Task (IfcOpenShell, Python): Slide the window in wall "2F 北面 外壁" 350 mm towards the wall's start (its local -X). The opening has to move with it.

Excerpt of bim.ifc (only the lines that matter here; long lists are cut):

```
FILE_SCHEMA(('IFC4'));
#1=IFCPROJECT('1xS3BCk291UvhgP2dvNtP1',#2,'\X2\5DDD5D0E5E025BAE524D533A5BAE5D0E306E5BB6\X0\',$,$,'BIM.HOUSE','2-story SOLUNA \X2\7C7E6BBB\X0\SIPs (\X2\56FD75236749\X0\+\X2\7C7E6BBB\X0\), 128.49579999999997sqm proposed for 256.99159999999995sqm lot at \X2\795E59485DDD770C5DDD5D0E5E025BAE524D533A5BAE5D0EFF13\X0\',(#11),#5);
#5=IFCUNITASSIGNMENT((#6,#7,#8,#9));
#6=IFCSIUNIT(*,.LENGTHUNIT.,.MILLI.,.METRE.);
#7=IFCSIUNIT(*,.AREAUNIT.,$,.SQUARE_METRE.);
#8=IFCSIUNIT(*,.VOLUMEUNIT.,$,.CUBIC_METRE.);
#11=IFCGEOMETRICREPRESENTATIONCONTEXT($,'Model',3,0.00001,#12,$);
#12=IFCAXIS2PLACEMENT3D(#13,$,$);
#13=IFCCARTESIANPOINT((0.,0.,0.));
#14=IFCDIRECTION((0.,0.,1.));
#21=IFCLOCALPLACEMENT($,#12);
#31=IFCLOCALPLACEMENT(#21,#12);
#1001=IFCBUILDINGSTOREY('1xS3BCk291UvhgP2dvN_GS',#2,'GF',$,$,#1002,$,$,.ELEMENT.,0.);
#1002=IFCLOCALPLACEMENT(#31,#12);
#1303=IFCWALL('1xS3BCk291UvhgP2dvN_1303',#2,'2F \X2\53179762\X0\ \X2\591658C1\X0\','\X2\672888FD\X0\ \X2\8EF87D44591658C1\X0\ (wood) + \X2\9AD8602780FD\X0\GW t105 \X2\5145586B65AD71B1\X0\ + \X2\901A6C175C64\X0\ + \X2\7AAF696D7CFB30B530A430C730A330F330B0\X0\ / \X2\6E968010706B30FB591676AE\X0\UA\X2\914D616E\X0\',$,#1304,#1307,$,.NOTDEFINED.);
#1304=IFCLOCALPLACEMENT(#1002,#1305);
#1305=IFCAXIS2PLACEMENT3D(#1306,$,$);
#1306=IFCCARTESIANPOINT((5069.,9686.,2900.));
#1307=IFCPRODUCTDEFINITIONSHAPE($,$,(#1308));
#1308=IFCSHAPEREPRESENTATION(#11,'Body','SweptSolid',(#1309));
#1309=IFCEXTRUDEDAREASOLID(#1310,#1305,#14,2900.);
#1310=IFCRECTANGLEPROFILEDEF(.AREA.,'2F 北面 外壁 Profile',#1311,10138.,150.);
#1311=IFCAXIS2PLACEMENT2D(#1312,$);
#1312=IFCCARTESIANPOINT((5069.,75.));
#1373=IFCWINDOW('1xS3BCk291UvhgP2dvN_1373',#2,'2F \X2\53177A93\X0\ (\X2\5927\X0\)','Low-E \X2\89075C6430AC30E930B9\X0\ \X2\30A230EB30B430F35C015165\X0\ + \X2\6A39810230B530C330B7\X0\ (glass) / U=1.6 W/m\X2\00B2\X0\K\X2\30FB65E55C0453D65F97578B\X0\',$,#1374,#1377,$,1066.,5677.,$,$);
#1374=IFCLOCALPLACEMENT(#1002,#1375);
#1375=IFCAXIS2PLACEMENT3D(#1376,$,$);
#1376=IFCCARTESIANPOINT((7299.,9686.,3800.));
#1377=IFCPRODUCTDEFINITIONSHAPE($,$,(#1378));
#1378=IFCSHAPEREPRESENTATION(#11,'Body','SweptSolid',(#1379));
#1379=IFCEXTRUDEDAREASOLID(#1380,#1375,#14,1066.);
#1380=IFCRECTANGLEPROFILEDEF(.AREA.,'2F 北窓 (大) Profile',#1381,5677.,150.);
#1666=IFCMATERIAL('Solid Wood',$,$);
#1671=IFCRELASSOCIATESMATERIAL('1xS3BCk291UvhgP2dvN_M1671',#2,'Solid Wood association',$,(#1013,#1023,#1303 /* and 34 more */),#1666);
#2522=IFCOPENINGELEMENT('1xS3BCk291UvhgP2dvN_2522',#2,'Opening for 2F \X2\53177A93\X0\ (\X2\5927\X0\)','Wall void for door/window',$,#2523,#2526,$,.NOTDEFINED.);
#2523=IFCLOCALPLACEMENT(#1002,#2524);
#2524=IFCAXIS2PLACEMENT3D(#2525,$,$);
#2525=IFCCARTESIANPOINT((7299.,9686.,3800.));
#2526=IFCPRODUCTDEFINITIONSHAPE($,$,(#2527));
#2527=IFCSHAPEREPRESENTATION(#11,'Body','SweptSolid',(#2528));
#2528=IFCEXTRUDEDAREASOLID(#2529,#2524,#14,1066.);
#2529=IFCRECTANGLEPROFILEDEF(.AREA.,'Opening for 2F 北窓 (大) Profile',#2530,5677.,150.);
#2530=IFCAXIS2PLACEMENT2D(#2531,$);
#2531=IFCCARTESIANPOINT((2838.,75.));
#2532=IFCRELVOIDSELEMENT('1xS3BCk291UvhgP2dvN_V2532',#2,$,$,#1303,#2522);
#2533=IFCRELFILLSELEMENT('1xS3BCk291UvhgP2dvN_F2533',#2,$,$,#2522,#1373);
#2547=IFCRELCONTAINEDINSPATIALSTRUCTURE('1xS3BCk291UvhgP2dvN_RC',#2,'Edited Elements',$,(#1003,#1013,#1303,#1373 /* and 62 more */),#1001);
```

```python
import ifcopenshell
import ifcopenshell.api.geometry
import ifcopenshell.util.placement

model = ifcopenshell.open("bim.ifc")

window = model.by_id(1373)
opening = window.FillsVoids[0].RelatingOpeningElement
wall = opening.VoidsElements[0].RelatingBuildingElement

wall_matrix = ifcopenshell.util.placement.get_local_placement(wall.ObjectPlacement)
shift = wall_matrix[:3, 0] * -350.0
before = ifcopenshell.util.placement.get_local_placement(window.ObjectPlacement)[:3, 3].copy()

# The window is not placed relative to its opening, so move both.
for product in (opening, window):
    matrix = ifcopenshell.util.placement.get_local_placement(product.ObjectPlacement)
    matrix[:3, 3] += shift
    ifcopenshell.api.geometry.edit_object_placement(model, product=product, matrix=matrix, is_si=False)

after = ifcopenshell.util.placement.get_local_placement(window.ObjectPlacement)[:3, 3]
print("window moved by", (after - before).round(3) + 0.0)

model.write("bim-out.ifc")
```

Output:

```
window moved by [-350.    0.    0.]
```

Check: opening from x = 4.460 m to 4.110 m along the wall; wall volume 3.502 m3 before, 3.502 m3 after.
